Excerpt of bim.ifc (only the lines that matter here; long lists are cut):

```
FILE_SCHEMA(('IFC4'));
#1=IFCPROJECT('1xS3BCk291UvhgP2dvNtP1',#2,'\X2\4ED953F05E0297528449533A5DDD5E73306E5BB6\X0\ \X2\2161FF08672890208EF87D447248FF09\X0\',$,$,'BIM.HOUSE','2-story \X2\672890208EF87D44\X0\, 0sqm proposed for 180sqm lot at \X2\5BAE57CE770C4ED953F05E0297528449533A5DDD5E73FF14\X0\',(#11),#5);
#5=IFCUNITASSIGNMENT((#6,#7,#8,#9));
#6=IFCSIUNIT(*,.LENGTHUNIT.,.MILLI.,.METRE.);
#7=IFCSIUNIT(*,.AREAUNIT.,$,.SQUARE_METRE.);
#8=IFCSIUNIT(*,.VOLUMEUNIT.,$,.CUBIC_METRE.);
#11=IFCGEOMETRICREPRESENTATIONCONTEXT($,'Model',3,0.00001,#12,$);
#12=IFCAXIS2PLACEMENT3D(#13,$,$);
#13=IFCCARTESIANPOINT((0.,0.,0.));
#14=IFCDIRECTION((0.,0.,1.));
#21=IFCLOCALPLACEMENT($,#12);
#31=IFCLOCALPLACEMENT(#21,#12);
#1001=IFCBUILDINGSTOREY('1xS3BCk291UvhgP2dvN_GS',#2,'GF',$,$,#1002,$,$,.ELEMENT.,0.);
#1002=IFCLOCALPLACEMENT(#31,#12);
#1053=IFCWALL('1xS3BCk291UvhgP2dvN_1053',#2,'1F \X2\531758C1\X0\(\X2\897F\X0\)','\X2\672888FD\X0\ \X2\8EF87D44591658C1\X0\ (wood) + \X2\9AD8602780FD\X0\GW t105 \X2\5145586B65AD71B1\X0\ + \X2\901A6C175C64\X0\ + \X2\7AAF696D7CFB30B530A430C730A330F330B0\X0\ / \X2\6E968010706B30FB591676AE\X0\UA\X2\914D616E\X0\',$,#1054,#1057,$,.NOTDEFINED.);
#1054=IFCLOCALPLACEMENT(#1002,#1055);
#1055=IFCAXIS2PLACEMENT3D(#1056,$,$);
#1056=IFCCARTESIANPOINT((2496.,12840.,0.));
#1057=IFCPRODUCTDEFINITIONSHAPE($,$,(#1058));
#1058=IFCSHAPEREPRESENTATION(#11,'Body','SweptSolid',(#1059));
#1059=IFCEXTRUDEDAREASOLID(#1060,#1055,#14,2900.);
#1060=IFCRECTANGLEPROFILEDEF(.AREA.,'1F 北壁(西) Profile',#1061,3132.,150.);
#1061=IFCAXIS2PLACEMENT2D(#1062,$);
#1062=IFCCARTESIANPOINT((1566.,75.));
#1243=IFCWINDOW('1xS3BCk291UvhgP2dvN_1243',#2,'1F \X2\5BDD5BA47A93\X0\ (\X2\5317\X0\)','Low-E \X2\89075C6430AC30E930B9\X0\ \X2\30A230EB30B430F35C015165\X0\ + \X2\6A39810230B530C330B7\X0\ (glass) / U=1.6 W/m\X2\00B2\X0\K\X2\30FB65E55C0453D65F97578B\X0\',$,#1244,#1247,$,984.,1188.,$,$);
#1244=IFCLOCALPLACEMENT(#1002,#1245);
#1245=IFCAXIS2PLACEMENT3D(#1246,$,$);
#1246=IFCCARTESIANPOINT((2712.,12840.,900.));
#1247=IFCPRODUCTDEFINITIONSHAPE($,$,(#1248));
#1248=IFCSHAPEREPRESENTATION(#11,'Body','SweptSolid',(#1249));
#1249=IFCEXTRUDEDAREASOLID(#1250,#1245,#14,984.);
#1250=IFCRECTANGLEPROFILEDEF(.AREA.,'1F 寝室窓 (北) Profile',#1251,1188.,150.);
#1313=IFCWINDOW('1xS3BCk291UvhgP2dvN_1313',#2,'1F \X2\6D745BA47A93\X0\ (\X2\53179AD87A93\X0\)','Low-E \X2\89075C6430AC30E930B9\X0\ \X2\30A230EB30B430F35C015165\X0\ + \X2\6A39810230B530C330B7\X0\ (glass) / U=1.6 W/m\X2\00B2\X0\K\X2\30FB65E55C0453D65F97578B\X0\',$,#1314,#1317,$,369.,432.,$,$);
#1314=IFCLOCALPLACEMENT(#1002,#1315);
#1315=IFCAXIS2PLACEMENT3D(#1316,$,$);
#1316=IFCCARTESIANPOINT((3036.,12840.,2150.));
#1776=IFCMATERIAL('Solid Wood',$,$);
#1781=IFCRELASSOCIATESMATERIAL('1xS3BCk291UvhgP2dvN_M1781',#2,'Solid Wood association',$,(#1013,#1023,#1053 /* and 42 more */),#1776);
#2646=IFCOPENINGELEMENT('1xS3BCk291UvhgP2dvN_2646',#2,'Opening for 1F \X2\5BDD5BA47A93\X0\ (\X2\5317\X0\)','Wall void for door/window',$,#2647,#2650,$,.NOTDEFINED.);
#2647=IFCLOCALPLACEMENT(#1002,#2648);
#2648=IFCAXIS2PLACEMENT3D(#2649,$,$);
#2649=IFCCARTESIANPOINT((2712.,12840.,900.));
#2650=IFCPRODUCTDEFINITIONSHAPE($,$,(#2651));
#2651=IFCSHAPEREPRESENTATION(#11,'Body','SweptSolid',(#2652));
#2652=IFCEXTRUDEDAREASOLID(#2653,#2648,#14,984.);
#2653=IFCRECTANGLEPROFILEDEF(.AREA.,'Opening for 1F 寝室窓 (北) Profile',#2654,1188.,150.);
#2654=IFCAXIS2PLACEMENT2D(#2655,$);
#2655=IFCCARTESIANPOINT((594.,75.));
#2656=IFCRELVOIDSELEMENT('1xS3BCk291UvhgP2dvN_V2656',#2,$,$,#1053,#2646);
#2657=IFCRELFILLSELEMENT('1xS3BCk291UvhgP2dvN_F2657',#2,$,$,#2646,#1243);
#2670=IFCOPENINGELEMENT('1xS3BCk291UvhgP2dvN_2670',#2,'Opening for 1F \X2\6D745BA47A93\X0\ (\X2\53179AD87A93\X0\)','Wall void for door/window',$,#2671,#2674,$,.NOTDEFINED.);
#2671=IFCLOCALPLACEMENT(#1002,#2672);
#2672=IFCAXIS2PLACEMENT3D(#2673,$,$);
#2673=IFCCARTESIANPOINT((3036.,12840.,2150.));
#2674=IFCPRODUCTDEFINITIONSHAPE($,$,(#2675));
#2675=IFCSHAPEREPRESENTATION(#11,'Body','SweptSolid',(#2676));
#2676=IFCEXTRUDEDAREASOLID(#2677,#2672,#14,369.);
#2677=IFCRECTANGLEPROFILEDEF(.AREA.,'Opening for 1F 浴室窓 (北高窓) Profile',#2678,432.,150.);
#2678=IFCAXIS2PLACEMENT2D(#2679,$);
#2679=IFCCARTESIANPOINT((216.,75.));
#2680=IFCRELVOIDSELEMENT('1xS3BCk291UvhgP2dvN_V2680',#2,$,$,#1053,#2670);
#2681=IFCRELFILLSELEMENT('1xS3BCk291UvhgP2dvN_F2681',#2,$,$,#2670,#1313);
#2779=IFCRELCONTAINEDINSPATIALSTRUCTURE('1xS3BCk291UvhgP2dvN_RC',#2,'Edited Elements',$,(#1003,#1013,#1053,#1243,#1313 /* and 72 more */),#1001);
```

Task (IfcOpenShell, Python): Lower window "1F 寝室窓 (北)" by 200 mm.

```python
import numpy as np
import ifcopenshell
import ifcopenshell.api.geometry
import ifcopenshell.util.placement
import ifcopenshell.util.unit

model = ifcopenshell.open("bim.ifc")
unit_scale = ifcopenshell.util.unit.calculate_unit_scale(model)

window = model.by_guid("1xS3BCk291UvhgP2dvN_1243")
opening = window.FillsVoids[0].RelatingOpeningElement
dz = -0.2 / unit_scale

shift = np.array([0.0, 0.0, dz])
# The window is not placed relative to its opening, so move both.
for product in (opening, window):
    matrix = ifcopenshell.util.placement.get_local_placement(product.ObjectPlacement)
    matrix[:3, 3] += shift
    ifcopenshell.api.geometry.edit_object_placement(model, product=product, matrix=matrix, is_si=False)

print(f"moved by {dz * unit_scale:+.3f} m")

model.write("bim_v2.ifc")
```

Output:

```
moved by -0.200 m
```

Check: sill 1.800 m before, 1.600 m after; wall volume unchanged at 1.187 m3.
